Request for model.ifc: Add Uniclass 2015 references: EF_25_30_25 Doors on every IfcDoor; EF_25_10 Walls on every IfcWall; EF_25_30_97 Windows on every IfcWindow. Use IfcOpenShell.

First a look at what the model holds.

```python
import ifcopenshell

model = ifcopenshell.open("model.ifc")
print(model.schema)
print("classifications:", [c.Name for c in model.by_type("IfcClassification")])
for ifc_class in ("IfcDoor", "IfcRoof", "IfcStair", "IfcWall", "IfcWindow"):
    print(ifc_class, len(model.by_type(ifc_class)))
```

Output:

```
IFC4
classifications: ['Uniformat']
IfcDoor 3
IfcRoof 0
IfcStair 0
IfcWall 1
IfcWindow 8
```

```python
import ifcopenshell
import ifcopenshell.api.classification

model = ifcopenshell.open("model.ifc")

system = ifcopenshell.api.classification.add_classification(model, classification="Uniclass 2015")

codes = {
    "IfcDoor": ("EF_25_30_25", "Doors"),
    "IfcWall": ("EF_25_10", "Walls"),
    "IfcWindow": ("EF_25_30_97", "Windows"),
}
for ifc_class, (code, name) in codes.items():
    products = model.by_type(ifc_class)
    ifcopenshell.api.classification.add_reference(
        model, products=products, classification=system, identification=code, name=name
    )
    print(code, len(products))

model.write("model_updated.ifc")
```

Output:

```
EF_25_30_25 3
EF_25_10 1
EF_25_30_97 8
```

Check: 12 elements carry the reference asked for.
